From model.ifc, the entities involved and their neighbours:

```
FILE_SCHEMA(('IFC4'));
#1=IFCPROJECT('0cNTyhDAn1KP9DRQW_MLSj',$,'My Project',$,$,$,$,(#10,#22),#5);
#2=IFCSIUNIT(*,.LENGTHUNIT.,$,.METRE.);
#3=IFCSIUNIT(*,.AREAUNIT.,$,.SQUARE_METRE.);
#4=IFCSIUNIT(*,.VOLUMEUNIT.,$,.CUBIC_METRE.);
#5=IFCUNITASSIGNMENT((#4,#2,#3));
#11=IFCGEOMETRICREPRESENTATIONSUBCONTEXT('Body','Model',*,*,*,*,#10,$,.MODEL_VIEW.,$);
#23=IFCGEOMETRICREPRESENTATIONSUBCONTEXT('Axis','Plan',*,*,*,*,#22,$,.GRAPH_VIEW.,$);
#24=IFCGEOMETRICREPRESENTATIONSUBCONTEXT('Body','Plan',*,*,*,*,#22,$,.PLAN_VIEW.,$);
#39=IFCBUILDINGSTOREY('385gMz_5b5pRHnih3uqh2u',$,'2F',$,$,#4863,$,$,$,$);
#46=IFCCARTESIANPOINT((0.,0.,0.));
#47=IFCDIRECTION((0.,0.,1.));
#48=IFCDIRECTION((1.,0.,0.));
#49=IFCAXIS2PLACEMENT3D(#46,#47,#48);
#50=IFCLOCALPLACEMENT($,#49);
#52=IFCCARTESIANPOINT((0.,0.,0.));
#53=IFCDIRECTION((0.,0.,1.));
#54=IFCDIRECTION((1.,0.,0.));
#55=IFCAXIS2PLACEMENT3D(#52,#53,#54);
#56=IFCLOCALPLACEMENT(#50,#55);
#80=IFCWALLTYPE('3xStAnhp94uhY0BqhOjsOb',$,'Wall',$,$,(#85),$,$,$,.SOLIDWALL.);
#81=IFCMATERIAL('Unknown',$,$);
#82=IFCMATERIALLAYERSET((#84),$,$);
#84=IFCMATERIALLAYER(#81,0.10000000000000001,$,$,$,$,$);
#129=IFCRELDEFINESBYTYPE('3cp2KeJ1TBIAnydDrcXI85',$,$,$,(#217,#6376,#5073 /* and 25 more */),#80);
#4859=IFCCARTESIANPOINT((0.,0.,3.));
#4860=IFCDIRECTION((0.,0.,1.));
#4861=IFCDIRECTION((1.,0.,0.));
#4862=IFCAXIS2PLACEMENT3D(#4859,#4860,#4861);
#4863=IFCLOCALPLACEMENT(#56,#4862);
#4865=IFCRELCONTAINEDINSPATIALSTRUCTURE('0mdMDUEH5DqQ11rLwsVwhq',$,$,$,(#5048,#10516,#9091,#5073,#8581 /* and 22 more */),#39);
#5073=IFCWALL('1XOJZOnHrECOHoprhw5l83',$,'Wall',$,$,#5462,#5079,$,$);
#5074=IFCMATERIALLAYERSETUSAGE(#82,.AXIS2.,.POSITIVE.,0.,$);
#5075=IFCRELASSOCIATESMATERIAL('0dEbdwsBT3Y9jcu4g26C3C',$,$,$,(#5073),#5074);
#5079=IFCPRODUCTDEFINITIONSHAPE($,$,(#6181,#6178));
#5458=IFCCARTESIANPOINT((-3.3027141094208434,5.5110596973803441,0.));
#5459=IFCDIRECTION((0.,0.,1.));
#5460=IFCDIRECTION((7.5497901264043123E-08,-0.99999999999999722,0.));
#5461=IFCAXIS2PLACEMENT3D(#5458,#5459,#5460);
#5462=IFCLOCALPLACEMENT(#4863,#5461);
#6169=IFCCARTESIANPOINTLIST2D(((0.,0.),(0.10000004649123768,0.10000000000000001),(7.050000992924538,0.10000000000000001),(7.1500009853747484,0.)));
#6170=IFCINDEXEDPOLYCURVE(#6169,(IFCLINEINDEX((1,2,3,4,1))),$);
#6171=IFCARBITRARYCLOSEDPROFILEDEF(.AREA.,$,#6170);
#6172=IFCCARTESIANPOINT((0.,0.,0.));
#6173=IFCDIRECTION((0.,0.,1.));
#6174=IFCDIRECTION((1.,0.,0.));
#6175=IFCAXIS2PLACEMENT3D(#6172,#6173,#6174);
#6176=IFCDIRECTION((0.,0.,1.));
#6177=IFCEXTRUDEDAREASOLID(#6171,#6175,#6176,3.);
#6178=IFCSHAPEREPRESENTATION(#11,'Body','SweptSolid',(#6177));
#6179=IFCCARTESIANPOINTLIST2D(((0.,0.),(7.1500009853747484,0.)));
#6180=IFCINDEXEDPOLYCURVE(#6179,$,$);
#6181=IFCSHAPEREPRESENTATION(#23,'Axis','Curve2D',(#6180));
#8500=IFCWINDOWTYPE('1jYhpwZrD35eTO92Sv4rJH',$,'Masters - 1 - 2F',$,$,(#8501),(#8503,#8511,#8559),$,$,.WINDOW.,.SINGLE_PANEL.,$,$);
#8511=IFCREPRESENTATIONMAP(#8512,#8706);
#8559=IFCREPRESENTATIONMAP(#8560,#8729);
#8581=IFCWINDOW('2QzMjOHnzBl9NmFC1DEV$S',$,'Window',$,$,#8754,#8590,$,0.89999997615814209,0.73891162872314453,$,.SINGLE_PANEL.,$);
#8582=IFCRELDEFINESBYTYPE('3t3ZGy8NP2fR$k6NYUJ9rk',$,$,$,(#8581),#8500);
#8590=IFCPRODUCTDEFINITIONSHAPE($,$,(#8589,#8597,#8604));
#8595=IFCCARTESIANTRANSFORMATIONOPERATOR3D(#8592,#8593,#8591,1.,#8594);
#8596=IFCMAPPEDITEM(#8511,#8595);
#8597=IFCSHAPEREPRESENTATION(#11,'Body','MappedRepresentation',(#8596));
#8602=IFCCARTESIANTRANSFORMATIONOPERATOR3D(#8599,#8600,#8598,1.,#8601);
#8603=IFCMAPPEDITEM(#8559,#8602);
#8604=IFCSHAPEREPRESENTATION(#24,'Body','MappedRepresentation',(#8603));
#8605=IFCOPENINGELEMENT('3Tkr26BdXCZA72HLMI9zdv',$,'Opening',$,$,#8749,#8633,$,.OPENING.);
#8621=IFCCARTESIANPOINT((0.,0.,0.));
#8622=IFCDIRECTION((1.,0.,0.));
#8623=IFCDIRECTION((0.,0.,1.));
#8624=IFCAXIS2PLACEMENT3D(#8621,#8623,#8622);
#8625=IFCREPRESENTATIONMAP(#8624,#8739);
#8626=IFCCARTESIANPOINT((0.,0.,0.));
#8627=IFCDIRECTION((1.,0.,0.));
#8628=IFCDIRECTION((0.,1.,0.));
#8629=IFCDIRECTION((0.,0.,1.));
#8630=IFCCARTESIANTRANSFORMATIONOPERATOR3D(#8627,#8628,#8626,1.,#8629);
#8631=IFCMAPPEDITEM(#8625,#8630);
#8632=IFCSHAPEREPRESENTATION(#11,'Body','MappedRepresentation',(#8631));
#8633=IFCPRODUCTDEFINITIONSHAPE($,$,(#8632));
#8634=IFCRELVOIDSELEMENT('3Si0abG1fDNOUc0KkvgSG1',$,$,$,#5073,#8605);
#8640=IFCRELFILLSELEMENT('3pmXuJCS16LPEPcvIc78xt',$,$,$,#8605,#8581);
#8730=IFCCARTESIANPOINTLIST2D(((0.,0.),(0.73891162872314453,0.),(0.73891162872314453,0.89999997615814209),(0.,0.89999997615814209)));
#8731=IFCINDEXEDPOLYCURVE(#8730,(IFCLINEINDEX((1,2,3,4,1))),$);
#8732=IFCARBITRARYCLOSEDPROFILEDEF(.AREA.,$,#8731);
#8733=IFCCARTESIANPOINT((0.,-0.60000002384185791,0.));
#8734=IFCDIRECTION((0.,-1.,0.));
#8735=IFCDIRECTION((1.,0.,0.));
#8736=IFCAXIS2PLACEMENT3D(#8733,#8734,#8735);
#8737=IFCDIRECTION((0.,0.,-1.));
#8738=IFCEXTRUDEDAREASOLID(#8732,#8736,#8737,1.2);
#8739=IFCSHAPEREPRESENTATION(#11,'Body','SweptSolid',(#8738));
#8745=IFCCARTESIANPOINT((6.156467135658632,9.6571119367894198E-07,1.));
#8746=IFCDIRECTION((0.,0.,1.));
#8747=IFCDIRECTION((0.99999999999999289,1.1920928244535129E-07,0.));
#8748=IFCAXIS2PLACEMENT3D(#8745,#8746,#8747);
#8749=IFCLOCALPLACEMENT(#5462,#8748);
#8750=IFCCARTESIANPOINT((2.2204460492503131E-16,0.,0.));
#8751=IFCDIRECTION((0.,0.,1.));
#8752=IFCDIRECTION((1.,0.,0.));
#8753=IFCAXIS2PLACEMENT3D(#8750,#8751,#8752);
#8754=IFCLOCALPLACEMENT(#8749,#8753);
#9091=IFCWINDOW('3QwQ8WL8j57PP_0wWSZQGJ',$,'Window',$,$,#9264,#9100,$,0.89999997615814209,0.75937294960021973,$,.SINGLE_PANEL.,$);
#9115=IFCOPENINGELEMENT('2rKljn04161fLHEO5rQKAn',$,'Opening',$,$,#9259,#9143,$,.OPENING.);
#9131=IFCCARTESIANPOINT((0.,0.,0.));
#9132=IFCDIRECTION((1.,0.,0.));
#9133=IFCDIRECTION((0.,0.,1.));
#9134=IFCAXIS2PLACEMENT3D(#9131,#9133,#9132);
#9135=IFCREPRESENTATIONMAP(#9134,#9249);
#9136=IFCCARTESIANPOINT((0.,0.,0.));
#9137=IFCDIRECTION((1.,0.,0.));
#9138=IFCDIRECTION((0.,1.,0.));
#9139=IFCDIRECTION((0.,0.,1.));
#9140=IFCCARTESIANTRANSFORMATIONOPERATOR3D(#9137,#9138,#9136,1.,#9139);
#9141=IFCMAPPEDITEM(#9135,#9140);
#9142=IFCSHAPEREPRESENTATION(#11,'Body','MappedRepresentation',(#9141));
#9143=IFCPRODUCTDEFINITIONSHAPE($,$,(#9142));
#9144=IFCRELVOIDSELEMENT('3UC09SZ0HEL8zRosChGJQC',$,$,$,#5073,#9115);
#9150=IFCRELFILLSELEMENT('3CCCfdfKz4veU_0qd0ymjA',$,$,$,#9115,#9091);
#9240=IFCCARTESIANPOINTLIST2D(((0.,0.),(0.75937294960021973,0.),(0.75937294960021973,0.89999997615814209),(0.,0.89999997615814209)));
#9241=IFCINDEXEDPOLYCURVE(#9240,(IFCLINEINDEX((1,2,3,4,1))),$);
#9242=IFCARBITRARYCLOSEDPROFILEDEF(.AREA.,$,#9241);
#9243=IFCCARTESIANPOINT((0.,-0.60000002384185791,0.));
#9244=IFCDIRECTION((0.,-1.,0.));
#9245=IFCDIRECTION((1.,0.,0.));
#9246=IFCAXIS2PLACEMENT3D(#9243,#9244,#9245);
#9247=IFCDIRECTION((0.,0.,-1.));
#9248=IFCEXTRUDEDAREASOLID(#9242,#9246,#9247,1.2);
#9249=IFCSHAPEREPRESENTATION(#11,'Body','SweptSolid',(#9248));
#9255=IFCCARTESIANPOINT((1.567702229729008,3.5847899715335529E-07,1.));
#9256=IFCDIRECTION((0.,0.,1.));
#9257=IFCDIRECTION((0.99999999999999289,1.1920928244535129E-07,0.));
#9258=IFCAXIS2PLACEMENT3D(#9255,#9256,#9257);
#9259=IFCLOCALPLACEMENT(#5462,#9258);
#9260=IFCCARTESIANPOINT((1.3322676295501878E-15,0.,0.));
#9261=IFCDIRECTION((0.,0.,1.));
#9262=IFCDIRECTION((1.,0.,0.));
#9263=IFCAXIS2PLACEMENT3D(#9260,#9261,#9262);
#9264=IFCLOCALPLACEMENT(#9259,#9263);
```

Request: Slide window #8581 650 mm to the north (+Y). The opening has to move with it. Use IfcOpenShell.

```python
import ifcopenshell
import ifcopenshell.api.geometry
import ifcopenshell.util.placement
import ifcopenshell.util.unit

model = ifcopenshell.open("model.ifc")
unit_scale = ifcopenshell.util.unit.calculate_unit_scale(model)

window = model.by_guid("2QzMjOHnzBl9NmFC1DEV$S")
opening = window.FillsVoids[0].RelatingOpeningElement
wall = opening.VoidsElements[0].RelatingBuildingElement

wall_matrix = ifcopenshell.util.placement.get_local_placement(wall.ObjectPlacement)
shift = wall_matrix[:3, 0] * -0.65 / unit_scale
before = ifcopenshell.util.placement.get_local_placement(window.ObjectPlacement)[:3, 3].copy()

# The window is placed relative to its opening, so it follows when the opening moves.
matrix = ifcopenshell.util.placement.get_local_placement(opening.ObjectPlacement)
matrix[:3, 3] += shift
ifcopenshell.api.geometry.edit_object_placement(
    model, product=opening, matrix=matrix, is_si=False, should_transform_children=True
)

after = ifcopenshell.util.placement.get_local_placement(window.ObjectPlacement)[:3, 3]
print("window moved by", (after - before).round(3) + 0.0)

model.write("model_rev.ifc")
```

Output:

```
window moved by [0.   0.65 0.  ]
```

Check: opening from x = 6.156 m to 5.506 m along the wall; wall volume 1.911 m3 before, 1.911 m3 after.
